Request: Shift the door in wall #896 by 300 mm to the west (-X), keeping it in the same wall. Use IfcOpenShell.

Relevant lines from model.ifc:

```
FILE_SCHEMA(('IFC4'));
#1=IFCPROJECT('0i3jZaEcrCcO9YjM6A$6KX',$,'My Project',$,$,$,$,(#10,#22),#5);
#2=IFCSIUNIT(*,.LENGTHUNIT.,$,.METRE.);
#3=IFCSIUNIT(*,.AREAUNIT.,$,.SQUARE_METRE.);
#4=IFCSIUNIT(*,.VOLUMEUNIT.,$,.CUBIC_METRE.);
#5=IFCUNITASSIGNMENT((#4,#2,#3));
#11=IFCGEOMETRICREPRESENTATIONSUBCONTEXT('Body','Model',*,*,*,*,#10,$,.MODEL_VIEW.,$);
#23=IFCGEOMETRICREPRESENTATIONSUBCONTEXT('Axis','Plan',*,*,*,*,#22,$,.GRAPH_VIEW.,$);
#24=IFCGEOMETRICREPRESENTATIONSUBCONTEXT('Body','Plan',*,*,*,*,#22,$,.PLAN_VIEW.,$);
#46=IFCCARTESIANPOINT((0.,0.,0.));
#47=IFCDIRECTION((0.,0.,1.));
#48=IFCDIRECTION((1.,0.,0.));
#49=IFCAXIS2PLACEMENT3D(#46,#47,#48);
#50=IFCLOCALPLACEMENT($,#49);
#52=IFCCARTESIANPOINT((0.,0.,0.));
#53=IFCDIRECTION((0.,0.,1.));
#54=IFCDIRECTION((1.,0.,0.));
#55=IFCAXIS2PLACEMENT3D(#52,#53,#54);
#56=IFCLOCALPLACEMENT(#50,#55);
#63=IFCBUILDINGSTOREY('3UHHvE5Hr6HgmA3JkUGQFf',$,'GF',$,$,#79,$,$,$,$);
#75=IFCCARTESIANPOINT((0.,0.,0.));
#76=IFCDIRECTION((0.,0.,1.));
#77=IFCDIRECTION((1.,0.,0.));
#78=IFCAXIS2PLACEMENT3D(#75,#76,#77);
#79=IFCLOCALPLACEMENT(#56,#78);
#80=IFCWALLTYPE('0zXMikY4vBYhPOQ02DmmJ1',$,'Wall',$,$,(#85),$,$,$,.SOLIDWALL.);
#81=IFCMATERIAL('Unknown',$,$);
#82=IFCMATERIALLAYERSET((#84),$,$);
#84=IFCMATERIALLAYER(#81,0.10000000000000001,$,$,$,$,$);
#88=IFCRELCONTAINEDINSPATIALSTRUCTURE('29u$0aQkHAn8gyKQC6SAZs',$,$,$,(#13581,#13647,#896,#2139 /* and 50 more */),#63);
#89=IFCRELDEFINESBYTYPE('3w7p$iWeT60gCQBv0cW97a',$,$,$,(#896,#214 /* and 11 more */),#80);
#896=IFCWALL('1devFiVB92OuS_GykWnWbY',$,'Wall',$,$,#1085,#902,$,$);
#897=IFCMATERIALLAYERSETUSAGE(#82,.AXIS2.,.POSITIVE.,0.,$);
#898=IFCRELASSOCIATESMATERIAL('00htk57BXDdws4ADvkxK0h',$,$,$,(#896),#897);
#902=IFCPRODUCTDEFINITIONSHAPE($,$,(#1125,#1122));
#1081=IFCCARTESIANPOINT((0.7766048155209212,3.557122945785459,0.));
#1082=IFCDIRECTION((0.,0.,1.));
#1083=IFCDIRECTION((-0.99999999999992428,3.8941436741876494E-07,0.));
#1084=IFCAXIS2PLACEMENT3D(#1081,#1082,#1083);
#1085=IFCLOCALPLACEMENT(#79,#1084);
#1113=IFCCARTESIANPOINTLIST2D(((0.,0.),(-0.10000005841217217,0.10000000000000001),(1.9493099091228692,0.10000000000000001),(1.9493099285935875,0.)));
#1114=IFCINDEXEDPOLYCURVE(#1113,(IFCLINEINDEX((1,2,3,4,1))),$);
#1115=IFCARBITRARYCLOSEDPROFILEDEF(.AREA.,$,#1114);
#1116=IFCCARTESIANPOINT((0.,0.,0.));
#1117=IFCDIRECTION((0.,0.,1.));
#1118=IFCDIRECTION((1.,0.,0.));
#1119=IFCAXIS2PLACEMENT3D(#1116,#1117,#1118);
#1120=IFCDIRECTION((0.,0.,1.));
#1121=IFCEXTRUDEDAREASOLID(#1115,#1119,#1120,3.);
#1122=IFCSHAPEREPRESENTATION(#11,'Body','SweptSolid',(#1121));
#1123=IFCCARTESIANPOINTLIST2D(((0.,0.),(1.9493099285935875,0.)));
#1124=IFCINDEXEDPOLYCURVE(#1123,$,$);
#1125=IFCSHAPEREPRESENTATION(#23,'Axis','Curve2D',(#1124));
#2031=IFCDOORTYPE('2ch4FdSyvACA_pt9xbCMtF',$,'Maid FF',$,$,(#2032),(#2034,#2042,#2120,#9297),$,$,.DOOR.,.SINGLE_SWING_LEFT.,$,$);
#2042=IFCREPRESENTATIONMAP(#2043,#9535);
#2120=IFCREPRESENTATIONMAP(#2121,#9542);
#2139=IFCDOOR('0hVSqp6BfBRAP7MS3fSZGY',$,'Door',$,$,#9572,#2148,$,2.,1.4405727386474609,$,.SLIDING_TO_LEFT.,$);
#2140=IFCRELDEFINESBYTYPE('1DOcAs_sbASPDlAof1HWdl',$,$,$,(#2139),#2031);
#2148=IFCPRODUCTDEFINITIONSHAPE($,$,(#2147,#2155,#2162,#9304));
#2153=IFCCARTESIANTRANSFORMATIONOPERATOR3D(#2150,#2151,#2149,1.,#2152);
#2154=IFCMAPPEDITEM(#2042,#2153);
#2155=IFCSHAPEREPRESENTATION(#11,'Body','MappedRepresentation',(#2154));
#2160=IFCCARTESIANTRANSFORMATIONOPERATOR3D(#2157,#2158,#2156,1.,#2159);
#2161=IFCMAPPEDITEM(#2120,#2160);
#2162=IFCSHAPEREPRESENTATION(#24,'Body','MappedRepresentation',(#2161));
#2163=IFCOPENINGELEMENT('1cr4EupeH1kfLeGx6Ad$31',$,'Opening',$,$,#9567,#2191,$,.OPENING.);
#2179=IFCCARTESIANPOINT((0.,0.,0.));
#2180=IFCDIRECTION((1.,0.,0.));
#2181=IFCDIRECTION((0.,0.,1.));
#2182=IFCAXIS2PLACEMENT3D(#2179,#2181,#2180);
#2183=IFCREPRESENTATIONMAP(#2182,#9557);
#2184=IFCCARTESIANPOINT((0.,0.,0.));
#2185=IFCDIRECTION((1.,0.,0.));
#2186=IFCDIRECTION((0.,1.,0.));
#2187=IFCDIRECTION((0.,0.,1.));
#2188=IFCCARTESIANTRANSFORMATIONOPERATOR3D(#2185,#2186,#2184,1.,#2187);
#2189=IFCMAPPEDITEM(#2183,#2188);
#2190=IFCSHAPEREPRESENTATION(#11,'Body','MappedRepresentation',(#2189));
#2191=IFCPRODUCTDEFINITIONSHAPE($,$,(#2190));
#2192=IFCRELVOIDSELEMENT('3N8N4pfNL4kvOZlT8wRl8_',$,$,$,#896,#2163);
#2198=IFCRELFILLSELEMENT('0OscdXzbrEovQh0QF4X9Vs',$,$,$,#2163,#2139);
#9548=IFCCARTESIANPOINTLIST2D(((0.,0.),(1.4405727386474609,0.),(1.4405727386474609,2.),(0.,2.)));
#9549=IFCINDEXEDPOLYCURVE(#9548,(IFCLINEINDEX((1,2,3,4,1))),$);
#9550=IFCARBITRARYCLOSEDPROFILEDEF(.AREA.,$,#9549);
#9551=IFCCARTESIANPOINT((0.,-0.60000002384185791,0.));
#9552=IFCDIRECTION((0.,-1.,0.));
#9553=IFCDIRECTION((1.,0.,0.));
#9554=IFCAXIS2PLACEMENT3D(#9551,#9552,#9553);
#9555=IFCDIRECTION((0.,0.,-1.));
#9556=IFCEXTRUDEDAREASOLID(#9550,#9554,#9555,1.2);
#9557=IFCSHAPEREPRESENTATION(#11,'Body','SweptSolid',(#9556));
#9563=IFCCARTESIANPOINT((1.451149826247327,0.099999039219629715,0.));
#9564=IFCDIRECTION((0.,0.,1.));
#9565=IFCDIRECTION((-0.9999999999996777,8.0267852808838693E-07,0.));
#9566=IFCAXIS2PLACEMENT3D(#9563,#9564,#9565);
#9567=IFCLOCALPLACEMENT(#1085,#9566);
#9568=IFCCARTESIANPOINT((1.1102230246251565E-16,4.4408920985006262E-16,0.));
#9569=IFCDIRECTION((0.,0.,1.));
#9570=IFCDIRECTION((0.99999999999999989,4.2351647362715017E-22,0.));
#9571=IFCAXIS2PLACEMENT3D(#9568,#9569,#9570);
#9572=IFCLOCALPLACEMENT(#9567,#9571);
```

```python
import ifcopenshell
import ifcopenshell.api.geometry
import ifcopenshell.util.placement
import ifcopenshell.util.unit

model = ifcopenshell.open("model.ifc")
unit_scale = ifcopenshell.util.unit.calculate_unit_scale(model)

door = model.by_guid("0hVSqp6BfBRAP7MS3fSZGY")
opening = door.FillsVoids[0].RelatingOpeningElement
wall = opening.VoidsElements[0].RelatingBuildingElement

wall_matrix = ifcopenshell.util.placement.get_local_placement(wall.ObjectPlacement)
shift = wall_matrix[:3, 0] * 0.3 / unit_scale
before = ifcopenshell.util.placement.get_local_placement(door.ObjectPlacement)[:3, 3].copy()

# The door is placed relative to its opening, so it follows when the opening moves.
matrix = ifcopenshell.util.placement.get_local_placement(opening.ObjectPlacement)
matrix[:3, 3] += shift
ifcopenshell.api.geometry.edit_object_placement(
    model, product=opening, matrix=matrix, is_si=False, should_transform_children=True
)

after = ifcopenshell.util.placement.get_local_placement(door.ObjectPlacement)[:3, 3]
print("door moved by", (after - before).round(3) + 0.0)

model.write("model-out.ifc")
```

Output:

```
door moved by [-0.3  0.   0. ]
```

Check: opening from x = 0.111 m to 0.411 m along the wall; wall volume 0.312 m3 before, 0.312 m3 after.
